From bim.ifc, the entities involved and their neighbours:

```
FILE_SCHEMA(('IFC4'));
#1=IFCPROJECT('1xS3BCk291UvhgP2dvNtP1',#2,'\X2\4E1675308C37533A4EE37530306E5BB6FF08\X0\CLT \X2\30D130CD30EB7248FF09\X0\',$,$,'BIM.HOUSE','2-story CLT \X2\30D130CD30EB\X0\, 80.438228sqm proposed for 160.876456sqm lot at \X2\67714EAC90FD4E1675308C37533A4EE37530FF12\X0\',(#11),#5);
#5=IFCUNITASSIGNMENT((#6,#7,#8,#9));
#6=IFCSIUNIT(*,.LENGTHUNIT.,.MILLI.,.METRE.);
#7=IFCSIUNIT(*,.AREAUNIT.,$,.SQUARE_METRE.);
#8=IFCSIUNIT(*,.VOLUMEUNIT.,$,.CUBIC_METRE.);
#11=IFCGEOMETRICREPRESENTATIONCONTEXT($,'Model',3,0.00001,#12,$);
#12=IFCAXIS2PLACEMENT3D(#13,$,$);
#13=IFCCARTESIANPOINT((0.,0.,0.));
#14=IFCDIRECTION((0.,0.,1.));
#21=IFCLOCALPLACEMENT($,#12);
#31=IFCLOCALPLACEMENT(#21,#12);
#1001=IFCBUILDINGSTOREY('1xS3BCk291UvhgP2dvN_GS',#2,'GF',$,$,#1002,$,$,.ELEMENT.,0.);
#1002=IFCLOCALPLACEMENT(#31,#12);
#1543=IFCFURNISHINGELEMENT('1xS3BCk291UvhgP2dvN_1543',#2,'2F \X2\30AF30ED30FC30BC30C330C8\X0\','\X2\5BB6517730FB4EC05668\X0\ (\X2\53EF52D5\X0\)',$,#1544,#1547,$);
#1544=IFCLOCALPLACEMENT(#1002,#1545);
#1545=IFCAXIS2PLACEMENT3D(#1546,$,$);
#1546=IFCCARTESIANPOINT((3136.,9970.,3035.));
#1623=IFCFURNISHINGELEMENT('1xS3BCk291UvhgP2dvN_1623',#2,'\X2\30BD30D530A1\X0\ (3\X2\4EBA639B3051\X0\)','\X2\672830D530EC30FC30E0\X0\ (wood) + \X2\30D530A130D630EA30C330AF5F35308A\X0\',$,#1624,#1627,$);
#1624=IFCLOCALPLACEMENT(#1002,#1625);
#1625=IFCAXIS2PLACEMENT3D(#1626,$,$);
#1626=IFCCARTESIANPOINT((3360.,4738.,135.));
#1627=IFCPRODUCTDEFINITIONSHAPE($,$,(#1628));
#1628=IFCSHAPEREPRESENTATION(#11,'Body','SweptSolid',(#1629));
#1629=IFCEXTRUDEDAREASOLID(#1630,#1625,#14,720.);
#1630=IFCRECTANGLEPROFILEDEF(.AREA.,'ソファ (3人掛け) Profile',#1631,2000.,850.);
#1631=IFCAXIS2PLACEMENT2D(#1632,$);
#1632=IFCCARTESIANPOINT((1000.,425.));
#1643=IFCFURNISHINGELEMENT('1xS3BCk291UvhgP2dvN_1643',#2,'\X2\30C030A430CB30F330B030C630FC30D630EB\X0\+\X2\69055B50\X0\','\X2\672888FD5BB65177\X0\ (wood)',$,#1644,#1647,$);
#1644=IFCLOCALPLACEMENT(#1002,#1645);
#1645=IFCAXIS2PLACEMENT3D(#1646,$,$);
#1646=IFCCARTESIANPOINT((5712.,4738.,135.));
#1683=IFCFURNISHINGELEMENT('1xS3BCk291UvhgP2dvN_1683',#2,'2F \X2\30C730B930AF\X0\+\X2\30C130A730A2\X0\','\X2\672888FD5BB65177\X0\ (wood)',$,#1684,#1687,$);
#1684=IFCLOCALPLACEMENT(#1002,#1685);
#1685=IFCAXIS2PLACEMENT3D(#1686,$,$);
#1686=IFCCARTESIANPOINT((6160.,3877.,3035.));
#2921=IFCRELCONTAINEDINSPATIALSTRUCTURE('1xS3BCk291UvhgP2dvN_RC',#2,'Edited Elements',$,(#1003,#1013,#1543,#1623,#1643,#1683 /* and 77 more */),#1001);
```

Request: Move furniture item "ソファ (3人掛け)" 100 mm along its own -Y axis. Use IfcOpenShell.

```python
import ifcopenshell
import ifcopenshell.api.geometry
import ifcopenshell.util.placement
import ifcopenshell.util.unit

model = ifcopenshell.open("bim.ifc")
unit_scale = ifcopenshell.util.unit.calculate_unit_scale(model)

item = model.by_guid("1xS3BCk291UvhgP2dvN_1623")
matrix = ifcopenshell.util.placement.get_local_placement(item.ObjectPlacement)
matrix[:3, 3] -= matrix[:3, 1] * 0.1 / unit_scale
ifcopenshell.api.geometry.edit_object_placement(model, product=item, matrix=matrix, is_si=False)

print(ifcopenshell.util.placement.get_local_placement(item.ObjectPlacement).round(3) + 0.0)

model.write("bim_rev.ifc")
```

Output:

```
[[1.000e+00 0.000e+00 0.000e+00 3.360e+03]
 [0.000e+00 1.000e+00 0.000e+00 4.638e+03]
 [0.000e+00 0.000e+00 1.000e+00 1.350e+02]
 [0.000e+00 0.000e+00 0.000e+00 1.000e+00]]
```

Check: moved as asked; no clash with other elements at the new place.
